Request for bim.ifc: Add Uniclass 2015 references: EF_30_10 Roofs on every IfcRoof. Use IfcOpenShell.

First a look at what the model holds.

```python
import ifcopenshell

model = ifcopenshell.open("bim.ifc")
print(model.schema)
print("classifications:", [c.Name for c in model.by_type("IfcClassification")])
for ifc_class in ("IfcDoor", "IfcRoof", "IfcStair", "IfcWall", "IfcWindow"):
    print(ifc_class, len(model.by_type(ifc_class)))
```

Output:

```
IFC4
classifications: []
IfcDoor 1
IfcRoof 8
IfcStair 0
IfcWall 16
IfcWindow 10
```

```python
import ifcopenshell
import ifcopenshell.api.classification

model = ifcopenshell.open("bim.ifc")

system = ifcopenshell.api.classification.add_classification(model, classification="Uniclass 2015")

codes = {
    "IfcRoof": ("EF_30_10", "Roofs"),
}
for ifc_class, (code, name) in codes.items():
    products = model.by_type(ifc_class)
    ifcopenshell.api.classification.add_reference(
        model, products=products, classification=system, identification=code, name=name
    )
    print(code, len(products))

model.write("bim_rev.ifc")
```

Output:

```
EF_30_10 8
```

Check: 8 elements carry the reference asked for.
